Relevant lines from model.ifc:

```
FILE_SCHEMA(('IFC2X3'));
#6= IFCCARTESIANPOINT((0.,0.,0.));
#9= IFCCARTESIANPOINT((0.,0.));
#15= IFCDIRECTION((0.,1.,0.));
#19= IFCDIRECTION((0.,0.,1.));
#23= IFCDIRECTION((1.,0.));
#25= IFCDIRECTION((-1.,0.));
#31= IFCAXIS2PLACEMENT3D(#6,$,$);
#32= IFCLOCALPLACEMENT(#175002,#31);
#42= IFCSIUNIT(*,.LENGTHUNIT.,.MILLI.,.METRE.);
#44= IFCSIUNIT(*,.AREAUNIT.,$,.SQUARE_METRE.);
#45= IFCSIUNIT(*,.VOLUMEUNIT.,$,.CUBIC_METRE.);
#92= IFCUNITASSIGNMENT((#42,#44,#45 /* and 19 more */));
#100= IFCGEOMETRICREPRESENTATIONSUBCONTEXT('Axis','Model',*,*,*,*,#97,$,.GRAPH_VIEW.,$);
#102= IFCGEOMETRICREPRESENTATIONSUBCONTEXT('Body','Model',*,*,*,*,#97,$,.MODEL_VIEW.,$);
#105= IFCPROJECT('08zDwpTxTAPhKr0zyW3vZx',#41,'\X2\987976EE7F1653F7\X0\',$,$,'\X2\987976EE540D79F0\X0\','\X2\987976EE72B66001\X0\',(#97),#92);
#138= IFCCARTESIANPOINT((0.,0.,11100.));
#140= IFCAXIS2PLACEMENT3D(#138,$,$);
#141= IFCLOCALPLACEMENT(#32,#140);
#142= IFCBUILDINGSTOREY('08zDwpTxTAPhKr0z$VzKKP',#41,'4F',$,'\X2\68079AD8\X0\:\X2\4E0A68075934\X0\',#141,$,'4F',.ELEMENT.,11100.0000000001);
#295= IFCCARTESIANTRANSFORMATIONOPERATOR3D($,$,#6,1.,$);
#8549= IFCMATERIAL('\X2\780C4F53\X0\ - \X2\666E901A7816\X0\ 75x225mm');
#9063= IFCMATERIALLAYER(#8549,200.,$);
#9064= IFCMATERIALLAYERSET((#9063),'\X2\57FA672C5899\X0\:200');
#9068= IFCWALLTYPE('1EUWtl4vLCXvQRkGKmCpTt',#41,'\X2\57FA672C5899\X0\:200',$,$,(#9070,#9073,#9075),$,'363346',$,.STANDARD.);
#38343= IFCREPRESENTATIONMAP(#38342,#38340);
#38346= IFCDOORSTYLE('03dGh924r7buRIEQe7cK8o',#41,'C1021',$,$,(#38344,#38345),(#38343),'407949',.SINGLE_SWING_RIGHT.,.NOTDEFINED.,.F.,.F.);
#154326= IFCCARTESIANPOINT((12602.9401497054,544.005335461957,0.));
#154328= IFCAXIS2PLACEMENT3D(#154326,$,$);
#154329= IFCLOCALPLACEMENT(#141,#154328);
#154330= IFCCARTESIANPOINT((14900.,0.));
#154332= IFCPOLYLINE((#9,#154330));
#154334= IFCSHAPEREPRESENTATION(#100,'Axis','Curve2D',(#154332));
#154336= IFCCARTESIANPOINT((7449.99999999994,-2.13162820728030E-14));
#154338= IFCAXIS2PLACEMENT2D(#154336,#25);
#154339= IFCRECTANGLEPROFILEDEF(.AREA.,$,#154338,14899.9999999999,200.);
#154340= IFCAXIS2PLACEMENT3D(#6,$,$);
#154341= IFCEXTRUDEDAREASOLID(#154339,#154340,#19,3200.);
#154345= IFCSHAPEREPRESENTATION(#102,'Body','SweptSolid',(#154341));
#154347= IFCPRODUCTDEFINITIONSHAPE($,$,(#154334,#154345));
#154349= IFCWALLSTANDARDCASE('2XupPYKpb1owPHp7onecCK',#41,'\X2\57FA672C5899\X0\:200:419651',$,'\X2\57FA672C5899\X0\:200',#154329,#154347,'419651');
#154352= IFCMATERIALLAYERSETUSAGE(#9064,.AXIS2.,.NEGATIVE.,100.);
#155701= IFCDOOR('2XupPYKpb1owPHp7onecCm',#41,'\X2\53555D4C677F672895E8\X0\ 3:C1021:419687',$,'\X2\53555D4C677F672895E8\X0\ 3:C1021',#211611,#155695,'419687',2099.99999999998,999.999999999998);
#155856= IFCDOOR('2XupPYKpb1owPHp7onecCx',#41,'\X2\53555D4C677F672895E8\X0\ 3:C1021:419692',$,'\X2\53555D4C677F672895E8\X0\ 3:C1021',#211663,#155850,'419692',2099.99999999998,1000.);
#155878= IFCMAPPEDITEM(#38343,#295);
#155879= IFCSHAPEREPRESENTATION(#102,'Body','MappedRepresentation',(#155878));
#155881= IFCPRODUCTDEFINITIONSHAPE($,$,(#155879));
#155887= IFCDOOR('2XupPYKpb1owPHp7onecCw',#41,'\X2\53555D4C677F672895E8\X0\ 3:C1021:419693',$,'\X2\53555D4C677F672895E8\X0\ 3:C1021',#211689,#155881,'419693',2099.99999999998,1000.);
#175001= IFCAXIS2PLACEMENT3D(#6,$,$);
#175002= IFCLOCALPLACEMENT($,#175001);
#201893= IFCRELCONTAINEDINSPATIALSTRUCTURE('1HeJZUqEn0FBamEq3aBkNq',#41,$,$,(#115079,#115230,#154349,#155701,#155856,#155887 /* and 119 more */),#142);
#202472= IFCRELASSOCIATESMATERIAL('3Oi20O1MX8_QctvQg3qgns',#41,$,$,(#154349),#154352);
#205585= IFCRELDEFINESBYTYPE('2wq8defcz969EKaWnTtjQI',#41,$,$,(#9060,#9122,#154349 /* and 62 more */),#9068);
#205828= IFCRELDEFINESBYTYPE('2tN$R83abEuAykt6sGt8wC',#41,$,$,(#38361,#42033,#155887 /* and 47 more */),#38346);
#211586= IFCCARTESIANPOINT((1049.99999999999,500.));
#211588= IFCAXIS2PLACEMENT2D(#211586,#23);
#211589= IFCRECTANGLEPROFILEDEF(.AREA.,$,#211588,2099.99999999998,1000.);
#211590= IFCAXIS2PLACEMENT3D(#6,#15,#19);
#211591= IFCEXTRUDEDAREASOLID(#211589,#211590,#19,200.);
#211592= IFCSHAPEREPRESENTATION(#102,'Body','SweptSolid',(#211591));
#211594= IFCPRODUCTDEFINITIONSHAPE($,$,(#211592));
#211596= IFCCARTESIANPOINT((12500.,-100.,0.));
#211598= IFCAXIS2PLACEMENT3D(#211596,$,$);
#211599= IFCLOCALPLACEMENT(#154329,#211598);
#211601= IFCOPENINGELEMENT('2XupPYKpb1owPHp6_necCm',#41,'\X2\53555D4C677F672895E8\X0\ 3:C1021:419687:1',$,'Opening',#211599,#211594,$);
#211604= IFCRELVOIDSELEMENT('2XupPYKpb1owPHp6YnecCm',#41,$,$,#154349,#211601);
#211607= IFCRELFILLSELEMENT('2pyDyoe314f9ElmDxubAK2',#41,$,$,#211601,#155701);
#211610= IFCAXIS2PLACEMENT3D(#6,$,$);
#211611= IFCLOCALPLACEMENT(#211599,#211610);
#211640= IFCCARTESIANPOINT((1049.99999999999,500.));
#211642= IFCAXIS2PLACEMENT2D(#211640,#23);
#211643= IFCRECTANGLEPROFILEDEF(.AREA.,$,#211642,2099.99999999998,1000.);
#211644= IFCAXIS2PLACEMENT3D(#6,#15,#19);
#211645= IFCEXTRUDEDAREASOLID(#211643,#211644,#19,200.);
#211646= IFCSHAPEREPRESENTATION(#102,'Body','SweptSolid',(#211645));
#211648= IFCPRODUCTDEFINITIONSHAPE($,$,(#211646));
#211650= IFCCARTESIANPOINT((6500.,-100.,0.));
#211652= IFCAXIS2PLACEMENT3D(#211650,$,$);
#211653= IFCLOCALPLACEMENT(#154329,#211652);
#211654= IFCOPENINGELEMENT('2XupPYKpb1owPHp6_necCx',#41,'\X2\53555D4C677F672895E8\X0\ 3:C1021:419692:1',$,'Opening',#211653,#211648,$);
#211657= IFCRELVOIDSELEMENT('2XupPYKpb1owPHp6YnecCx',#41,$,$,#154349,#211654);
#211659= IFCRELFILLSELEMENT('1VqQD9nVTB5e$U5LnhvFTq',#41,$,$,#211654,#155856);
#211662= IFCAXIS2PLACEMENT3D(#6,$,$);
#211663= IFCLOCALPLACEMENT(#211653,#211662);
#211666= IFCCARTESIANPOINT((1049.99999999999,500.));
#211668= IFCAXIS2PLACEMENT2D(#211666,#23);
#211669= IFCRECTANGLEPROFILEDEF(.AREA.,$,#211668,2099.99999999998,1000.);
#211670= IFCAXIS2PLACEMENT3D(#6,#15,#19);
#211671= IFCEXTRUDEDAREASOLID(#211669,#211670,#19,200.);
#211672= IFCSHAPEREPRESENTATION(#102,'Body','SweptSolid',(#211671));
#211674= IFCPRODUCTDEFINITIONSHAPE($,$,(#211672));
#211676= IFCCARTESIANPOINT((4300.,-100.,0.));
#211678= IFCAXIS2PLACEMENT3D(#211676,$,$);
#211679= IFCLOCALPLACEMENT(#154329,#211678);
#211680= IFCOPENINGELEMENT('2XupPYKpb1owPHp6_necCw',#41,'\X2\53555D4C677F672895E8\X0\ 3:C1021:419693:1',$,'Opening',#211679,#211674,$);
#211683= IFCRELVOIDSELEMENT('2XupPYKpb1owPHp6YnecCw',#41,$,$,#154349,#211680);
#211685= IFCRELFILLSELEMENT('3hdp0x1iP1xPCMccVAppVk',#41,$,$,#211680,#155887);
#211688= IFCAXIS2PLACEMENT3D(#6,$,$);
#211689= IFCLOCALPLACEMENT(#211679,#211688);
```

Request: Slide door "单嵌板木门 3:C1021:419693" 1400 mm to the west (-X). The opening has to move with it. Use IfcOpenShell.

```python
import ifcopenshell
import ifcopenshell.api.geometry
import ifcopenshell.util.placement

model = ifcopenshell.open("model.ifc")

door = model.by_guid("2XupPYKpb1owPHp7onecCw")
opening = door.FillsVoids[0].RelatingOpeningElement
wall = opening.VoidsElements[0].RelatingBuildingElement

wall_matrix = ifcopenshell.util.placement.get_local_placement(wall.ObjectPlacement)
shift = wall_matrix[:3, 0] * -1400.0
before = ifcopenshell.util.placement.get_local_placement(door.ObjectPlacement)[:3, 3].copy()

# The door is placed relative to its opening, so it follows when the opening moves.
matrix = ifcopenshell.util.placement.get_local_placement(opening.ObjectPlacement)
matrix[:3, 3] += shift
ifcopenshell.api.geometry.edit_object_placement(
    model, product=opening, matrix=matrix, is_si=False, should_transform_children=True
)

after = ifcopenshell.util.placement.get_local_placement(door.ObjectPlacement)[:3, 3]
print("door moved by", (after - before).round(3) + 0.0)

model.write("model_updated.ifc")
```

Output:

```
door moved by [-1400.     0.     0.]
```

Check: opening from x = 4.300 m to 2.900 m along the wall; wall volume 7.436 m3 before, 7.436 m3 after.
